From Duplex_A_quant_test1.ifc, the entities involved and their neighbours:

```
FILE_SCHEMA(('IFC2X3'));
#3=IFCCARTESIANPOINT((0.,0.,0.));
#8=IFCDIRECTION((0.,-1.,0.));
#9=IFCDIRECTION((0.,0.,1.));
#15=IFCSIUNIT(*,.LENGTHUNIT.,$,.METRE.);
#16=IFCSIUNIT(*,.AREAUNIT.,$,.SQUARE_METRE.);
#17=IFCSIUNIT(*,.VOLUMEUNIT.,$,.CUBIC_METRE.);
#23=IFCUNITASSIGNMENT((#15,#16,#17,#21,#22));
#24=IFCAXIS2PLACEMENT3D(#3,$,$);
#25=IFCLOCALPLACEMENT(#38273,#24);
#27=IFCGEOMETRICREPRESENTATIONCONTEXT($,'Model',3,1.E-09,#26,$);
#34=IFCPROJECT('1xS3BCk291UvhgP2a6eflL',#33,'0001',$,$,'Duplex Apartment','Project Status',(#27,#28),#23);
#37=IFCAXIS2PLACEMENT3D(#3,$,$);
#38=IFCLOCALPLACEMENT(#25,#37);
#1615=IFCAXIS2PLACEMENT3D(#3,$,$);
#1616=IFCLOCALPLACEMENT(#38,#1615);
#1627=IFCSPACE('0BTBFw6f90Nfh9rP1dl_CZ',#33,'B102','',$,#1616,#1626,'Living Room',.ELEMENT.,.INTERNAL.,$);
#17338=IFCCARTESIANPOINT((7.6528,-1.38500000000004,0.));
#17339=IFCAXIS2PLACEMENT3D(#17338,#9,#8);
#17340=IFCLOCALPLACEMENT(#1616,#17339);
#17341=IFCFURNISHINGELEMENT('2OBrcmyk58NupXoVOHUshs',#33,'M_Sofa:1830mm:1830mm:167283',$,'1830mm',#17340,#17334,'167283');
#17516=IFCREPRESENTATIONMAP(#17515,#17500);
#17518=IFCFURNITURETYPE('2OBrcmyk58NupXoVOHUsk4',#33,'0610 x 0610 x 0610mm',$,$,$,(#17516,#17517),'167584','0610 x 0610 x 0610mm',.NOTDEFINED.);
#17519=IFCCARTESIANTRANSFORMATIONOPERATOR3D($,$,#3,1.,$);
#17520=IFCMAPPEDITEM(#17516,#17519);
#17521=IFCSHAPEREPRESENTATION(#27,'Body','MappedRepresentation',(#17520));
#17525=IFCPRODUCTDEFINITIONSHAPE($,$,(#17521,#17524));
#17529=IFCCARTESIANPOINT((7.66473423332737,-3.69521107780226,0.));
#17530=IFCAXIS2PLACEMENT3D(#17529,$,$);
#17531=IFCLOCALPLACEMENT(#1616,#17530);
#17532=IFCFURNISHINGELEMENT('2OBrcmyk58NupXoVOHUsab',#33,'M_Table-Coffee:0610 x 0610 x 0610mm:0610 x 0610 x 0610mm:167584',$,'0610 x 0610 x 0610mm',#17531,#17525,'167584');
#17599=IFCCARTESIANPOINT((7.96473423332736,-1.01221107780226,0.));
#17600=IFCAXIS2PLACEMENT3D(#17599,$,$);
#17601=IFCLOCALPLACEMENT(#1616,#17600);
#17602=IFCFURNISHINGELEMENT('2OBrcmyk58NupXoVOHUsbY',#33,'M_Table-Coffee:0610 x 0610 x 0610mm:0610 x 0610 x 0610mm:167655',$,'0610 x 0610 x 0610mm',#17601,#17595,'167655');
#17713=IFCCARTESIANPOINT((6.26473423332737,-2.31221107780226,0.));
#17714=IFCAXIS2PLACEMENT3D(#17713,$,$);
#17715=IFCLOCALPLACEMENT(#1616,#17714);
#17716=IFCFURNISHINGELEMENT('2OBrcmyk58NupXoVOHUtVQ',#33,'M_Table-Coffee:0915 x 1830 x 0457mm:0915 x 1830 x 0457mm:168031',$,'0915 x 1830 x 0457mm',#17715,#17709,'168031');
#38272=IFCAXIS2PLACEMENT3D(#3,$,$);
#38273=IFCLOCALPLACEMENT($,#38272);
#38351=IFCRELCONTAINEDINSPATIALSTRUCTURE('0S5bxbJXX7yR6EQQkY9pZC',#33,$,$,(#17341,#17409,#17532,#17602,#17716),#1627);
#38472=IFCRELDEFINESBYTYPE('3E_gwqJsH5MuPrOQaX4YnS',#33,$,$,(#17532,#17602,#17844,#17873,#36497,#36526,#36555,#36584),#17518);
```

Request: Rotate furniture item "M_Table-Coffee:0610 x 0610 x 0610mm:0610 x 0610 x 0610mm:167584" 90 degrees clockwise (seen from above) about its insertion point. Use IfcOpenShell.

```python
import ifcopenshell
import ifcopenshell.api.geometry
import ifcopenshell.util.placement

model = ifcopenshell.open("Duplex_A_quant_test1.ifc")

item = model.by_id(17532)
matrix = ifcopenshell.util.placement.get_local_placement(item.ObjectPlacement)
matrix = matrix @ ifcopenshell.util.placement.rotation(-90, "Z")
ifcopenshell.api.geometry.edit_object_placement(model, product=item, matrix=matrix, is_si=False)

print(ifcopenshell.util.placement.get_local_placement(item.ObjectPlacement).round(3) + 0.0)

model.write("Duplex_A_quant_test1_v2.ifc")
```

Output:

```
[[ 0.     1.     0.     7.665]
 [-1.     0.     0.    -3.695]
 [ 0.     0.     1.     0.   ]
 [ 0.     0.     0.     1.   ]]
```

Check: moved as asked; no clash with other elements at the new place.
